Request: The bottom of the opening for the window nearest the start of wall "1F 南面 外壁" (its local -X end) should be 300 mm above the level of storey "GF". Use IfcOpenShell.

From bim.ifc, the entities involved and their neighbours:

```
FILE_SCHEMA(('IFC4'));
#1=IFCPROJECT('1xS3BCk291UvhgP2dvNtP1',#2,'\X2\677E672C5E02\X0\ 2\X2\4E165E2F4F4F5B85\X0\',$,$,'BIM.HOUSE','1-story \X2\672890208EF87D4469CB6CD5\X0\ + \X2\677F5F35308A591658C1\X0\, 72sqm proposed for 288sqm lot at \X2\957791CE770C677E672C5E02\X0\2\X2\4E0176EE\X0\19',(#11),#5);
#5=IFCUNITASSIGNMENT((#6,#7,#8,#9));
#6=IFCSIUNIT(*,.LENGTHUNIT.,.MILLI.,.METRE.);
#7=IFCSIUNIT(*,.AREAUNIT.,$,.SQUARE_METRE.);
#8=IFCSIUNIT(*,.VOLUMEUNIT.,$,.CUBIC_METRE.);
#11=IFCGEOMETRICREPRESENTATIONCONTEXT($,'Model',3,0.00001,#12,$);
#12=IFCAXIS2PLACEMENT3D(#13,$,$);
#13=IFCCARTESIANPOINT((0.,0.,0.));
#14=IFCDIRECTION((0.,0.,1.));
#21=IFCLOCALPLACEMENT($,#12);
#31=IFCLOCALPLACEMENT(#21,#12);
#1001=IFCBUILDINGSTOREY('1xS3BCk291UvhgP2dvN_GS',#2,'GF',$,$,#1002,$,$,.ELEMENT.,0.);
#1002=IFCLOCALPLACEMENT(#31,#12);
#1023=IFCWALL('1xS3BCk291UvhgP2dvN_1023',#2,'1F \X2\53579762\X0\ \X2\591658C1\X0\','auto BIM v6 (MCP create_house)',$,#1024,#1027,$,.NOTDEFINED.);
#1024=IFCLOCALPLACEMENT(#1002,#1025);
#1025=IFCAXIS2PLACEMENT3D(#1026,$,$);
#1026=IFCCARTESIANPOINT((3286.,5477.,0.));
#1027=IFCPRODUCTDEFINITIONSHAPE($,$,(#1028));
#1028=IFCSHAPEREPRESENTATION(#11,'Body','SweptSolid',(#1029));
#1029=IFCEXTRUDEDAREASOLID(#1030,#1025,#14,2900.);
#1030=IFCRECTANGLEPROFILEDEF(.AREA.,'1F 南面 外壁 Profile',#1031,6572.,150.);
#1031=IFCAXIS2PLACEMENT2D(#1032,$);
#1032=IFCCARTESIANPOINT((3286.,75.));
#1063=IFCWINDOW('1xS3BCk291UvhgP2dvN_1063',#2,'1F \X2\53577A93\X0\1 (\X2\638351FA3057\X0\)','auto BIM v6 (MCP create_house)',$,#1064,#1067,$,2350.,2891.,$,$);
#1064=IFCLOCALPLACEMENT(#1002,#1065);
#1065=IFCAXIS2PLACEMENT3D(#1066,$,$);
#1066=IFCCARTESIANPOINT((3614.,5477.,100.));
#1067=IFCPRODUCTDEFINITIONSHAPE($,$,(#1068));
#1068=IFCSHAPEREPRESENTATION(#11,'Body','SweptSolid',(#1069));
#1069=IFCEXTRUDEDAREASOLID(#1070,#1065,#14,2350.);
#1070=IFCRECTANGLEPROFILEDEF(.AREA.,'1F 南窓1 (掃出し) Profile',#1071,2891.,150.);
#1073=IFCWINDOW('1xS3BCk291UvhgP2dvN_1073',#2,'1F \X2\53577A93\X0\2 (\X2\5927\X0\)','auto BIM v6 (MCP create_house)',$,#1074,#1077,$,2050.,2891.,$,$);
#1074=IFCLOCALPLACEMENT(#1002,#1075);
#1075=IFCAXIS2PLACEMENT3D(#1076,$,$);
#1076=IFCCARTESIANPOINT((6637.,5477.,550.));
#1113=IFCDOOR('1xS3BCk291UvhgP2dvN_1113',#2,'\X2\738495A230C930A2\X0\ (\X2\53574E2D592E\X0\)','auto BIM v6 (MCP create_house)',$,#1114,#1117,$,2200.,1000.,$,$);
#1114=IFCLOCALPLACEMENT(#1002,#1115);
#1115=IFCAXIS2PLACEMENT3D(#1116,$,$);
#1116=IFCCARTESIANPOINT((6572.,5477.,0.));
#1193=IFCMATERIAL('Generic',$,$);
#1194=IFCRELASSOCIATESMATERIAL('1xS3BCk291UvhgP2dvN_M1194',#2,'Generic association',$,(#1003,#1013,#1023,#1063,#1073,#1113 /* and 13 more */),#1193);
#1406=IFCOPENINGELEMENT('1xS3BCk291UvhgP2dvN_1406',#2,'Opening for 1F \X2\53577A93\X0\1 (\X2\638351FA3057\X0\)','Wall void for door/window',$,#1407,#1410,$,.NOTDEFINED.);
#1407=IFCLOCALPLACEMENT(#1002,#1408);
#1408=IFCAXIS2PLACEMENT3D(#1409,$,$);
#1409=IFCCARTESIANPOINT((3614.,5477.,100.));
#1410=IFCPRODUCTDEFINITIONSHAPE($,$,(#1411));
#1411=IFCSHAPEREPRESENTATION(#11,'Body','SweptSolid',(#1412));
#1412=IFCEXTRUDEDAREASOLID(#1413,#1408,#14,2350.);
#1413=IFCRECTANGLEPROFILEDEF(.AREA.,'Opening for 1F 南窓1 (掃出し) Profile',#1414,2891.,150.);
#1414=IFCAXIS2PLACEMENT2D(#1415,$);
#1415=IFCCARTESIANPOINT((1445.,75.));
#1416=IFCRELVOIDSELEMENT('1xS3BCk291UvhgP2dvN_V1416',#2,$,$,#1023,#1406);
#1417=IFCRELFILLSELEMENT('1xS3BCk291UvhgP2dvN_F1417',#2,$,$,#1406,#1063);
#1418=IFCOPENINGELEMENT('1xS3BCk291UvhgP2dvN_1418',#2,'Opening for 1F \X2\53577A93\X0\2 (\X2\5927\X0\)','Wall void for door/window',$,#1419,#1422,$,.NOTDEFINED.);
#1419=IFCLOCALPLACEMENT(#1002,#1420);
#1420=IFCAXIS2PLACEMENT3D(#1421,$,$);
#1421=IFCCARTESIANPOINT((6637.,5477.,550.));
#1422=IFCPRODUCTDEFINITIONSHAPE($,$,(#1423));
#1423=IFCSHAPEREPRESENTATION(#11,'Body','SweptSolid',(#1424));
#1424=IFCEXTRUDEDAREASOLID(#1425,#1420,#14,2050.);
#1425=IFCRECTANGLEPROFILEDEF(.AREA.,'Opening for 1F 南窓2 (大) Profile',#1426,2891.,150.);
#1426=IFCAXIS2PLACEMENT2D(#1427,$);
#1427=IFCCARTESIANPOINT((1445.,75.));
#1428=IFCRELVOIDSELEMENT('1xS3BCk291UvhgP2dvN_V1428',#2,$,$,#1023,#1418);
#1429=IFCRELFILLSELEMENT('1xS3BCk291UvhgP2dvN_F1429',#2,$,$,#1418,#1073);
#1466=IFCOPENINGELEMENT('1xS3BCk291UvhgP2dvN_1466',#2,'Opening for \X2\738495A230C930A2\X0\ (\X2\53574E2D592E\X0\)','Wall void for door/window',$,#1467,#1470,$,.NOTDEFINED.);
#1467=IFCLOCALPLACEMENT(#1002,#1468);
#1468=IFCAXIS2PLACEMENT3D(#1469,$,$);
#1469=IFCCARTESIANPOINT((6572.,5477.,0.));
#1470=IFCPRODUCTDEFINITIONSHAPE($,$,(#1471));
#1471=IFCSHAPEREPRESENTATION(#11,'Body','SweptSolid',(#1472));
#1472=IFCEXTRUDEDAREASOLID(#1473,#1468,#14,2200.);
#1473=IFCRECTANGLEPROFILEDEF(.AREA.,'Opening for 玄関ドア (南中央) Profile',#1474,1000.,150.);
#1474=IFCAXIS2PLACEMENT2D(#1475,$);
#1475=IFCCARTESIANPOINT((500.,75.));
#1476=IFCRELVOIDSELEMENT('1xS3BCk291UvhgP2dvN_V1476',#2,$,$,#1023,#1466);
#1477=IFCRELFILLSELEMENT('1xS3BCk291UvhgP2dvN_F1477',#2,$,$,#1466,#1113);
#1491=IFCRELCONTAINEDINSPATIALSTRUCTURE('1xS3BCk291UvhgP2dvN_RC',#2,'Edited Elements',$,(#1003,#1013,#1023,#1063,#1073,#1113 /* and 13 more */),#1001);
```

```python
import numpy as np
import ifcopenshell
import ifcopenshell.api.geometry
import ifcopenshell.geom
import ifcopenshell.util.element
import ifcopenshell.util.placement
import ifcopenshell.util.shape
import ifcopenshell.util.unit

model = ifcopenshell.open("bim.ifc")
unit_scale = ifcopenshell.util.unit.calculate_unit_scale(model)

window = model.by_guid("1xS3BCk291UvhgP2dvN_1063")
opening = window.FillsVoids[0].RelatingOpeningElement
storey = ifcopenshell.util.element.get_container(window, ifc_class="IfcBuildingStorey")
level = ifcopenshell.util.placement.get_local_placement(storey.ObjectPlacement)[2, 3]

# The opening's origin need not be at the sill, so measure its lowest point.
shape = ifcopenshell.geom.create_shape(ifcopenshell.geom.settings(), opening)
bottom = ifcopenshell.util.shape.get_shape_bottom_elevation(shape, shape.geometry) / unit_scale
dz = level + 0.3 / unit_scale - bottom

shift = np.array([0.0, 0.0, dz])
# The window is not placed relative to its opening, so move both.
for product in (opening, window):
    matrix = ifcopenshell.util.placement.get_local_placement(product.ObjectPlacement)
    matrix[:3, 3] += shift
    ifcopenshell.api.geometry.edit_object_placement(model, product=product, matrix=matrix, is_si=False)

print(f"moved by {dz * unit_scale:+.3f} m")

model.write("bim_updated.ifc")
```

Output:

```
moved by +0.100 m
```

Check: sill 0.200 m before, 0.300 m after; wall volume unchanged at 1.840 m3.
